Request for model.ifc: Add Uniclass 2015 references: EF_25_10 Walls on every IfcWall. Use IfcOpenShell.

First a look at what the model holds.

```python
import ifcopenshell

model = ifcopenshell.open("model.ifc")
print(model.schema)
print("classifications:", [c.Name for c in model.by_type("IfcClassification")])
for ifc_class in ("IfcDoor", "IfcRoof", "IfcStair", "IfcWall", "IfcWindow"):
    print(ifc_class, len(model.by_type(ifc_class)))
```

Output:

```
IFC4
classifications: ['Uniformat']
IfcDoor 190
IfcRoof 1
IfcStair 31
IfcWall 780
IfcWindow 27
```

```python
import ifcopenshell
import ifcopenshell.api.classification

model = ifcopenshell.open("model.ifc")

system = ifcopenshell.api.classification.add_classification(model, classification="Uniclass 2015")

codes = {
    "IfcWall": ("EF_25_10", "Walls"),
}
for ifc_class, (code, name) in codes.items():
    products = model.by_type(ifc_class)
    ifcopenshell.api.classification.add_reference(
        model, products=products, classification=system, identification=code, name=name
    )
    print(code, len(products))

model.write("model_v2.ifc")
```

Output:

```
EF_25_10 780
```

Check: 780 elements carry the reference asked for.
